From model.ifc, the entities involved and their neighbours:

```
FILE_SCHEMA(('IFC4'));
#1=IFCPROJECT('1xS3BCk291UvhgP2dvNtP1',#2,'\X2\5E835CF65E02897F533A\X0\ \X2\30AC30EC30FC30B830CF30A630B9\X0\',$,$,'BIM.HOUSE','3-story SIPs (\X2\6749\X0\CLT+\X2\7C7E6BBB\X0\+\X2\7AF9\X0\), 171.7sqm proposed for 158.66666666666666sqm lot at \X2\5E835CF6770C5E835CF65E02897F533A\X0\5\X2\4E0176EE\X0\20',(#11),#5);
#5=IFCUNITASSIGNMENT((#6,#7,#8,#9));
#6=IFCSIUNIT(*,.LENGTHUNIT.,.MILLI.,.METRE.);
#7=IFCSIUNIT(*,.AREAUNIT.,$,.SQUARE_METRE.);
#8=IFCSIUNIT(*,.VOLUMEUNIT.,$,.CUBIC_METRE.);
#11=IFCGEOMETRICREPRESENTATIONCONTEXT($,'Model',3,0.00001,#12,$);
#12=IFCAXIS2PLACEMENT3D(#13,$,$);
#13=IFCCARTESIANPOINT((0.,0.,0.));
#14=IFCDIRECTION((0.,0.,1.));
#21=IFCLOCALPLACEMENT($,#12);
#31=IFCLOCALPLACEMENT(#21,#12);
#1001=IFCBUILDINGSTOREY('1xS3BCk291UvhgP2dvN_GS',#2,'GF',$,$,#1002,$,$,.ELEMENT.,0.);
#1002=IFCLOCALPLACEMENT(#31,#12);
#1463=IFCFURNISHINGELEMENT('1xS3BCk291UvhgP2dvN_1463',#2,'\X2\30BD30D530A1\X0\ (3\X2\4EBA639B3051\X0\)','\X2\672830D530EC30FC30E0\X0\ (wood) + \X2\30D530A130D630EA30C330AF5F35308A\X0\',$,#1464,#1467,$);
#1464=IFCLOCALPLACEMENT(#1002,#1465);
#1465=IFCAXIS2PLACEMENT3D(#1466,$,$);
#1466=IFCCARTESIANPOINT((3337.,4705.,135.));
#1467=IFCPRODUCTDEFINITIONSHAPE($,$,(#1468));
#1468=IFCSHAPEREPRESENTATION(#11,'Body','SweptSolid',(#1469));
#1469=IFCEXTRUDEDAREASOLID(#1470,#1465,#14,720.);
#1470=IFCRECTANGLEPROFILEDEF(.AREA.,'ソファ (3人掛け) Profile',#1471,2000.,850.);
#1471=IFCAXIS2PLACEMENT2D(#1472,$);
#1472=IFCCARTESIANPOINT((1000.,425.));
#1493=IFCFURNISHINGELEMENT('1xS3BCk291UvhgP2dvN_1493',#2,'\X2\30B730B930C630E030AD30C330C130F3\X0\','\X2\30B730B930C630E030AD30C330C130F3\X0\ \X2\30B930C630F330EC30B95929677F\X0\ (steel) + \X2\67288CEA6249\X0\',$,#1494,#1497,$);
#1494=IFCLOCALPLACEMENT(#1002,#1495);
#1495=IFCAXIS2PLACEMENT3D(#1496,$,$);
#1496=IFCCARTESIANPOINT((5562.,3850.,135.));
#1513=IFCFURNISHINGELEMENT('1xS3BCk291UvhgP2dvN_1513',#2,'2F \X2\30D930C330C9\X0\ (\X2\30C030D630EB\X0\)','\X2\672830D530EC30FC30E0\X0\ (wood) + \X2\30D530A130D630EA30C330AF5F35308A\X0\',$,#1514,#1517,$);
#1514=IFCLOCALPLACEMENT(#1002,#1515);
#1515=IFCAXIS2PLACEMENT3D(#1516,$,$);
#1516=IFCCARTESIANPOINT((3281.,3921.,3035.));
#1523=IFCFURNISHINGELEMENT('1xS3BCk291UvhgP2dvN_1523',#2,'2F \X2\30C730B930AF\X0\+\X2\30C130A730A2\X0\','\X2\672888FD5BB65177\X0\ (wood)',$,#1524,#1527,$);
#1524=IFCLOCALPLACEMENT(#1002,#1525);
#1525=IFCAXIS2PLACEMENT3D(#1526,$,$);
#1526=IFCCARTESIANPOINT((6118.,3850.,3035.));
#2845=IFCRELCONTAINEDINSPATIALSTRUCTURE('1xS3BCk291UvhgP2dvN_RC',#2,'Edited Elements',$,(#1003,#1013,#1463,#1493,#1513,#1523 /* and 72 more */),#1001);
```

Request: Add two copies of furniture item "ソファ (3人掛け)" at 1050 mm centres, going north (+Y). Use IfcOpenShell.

```python
import numpy as np
import ifcopenshell
import ifcopenshell.api.geometry
import ifcopenshell.api.root
import ifcopenshell.util.element
import ifcopenshell.util.placement
import ifcopenshell.util.unit

model = ifcopenshell.open("model.ifc")
unit_scale = ifcopenshell.util.unit.calculate_unit_scale(model)


def reuse_history(source, copy):
    """copy_class also copies each property set's owner history, people and application; keep the originals."""
    for rel in copy.IsDefinedBy:
        if rel.is_a("IfcRelDefinesByProperties") and (history := rel.RelatingPropertyDefinition.OwnerHistory):
            rel.RelatingPropertyDefinition.OwnerHistory = source.OwnerHistory
            ifcopenshell.util.element.remove_deep2(model, history)


source = model.by_guid("1xS3BCk291UvhgP2dvN_1463")
base = ifcopenshell.util.placement.get_local_placement(source.ObjectPlacement)
step = np.array([0.0, 1.0, 0.0]) * 1.05 / unit_scale

for i in range(1, 3):
    copy = ifcopenshell.api.root.copy_class(model, product=source)
    copy.Representation = ifcopenshell.util.element.copy_deep(
        model, source.Representation, exclude=["IfcGeometricRepresentationContext", "IfcRepresentationMap"]
    )
    reuse_history(source, copy)
    matrix = base.copy()
    matrix[:3, 3] += i * step
    print("added at", matrix[:3, 3].round(3) + 0.0)
    ifcopenshell.api.geometry.edit_object_placement(model, product=copy, matrix=matrix, is_si=False)

model.write("model_rev.ifc")
```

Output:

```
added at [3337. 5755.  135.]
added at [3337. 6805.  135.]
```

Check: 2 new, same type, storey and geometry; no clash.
